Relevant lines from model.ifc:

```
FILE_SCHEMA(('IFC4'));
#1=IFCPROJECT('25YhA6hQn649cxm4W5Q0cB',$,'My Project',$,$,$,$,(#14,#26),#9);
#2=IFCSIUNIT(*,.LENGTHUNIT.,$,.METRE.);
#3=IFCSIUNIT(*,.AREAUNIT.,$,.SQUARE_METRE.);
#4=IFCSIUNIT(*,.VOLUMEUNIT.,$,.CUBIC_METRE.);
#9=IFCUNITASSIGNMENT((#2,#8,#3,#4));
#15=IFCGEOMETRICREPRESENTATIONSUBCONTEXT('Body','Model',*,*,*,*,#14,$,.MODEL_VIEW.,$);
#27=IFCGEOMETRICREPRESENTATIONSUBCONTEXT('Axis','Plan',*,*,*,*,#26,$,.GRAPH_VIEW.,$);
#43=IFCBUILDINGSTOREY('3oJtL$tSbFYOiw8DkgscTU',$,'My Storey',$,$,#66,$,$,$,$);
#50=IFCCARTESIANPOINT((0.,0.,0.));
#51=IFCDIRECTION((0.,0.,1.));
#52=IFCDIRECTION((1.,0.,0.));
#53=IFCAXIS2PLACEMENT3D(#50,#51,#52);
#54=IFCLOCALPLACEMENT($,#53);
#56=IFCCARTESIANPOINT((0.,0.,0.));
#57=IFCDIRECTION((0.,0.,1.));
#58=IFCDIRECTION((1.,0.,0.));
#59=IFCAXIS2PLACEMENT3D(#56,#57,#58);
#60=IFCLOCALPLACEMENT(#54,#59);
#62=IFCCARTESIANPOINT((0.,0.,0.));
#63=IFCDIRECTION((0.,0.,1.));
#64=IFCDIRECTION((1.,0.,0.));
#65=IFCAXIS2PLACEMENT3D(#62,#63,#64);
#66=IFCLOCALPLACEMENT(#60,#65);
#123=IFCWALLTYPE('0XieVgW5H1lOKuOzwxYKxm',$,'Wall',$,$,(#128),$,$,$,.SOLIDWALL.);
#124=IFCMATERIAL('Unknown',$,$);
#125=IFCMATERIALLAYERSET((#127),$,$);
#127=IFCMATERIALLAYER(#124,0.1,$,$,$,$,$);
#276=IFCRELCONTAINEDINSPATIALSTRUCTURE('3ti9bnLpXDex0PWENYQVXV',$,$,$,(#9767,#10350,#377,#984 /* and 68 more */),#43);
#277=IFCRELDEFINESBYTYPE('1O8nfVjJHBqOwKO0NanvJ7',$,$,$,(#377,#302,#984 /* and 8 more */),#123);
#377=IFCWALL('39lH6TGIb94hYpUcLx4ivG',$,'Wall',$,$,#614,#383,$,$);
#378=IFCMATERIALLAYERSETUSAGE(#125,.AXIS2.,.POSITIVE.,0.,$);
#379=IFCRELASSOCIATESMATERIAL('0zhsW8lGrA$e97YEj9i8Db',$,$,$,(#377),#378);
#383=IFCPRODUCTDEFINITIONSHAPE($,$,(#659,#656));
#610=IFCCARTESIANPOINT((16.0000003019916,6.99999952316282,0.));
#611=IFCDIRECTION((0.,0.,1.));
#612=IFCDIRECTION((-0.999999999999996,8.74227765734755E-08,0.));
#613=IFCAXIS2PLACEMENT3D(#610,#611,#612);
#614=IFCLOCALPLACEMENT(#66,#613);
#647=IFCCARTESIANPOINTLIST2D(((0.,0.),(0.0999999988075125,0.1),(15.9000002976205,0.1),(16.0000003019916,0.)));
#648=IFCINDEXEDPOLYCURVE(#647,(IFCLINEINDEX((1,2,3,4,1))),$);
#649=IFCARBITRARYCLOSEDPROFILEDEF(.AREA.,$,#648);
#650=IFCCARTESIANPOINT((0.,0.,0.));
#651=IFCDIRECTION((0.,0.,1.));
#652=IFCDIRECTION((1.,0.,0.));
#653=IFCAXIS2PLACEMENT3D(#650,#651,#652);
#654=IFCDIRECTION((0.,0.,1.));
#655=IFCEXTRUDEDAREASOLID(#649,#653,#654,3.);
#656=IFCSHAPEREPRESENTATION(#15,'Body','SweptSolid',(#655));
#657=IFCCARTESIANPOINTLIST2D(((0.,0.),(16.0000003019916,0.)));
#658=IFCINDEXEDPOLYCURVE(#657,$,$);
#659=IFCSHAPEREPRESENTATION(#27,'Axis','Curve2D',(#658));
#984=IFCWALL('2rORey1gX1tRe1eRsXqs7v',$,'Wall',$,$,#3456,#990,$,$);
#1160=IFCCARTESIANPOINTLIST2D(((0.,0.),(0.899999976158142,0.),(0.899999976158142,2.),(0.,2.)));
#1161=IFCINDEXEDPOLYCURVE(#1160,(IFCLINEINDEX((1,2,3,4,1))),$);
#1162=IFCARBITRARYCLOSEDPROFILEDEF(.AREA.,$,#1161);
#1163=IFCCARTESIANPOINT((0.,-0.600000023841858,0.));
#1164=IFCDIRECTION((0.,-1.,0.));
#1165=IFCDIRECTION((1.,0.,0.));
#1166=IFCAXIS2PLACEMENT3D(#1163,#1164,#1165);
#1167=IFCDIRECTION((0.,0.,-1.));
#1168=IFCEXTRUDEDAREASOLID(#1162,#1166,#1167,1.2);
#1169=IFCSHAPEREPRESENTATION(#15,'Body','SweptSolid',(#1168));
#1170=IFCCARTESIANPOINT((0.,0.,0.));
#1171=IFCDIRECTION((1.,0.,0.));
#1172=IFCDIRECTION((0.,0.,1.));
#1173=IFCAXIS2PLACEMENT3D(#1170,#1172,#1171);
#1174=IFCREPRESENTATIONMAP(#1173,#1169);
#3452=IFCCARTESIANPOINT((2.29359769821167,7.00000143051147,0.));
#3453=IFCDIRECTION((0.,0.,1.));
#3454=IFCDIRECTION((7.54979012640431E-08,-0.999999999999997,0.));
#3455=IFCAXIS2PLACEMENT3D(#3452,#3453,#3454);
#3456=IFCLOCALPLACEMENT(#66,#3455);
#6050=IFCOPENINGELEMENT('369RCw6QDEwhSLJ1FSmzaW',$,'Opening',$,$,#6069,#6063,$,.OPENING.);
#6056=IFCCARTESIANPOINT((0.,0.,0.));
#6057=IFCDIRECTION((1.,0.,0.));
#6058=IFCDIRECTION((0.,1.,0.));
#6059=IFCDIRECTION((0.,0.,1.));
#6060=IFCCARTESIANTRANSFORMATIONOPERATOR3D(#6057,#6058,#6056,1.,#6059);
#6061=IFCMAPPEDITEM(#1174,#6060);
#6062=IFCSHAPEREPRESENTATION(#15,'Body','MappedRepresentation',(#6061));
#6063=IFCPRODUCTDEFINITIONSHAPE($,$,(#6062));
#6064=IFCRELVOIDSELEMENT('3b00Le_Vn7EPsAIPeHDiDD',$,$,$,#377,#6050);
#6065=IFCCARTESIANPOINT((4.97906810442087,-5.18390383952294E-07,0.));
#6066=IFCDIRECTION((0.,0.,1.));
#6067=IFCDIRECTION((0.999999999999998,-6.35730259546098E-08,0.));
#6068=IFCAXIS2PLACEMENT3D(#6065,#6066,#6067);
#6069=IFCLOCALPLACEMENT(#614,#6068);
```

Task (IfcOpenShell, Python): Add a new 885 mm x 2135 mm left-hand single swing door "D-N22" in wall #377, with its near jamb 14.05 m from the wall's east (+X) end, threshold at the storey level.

```python
import numpy as np
import ifcopenshell
import ifcopenshell.api.feature
import ifcopenshell.api.geometry
import ifcopenshell.api.root
import ifcopenshell.api.spatial
import ifcopenshell.geom
import ifcopenshell.util.element
import ifcopenshell.util.placement
import ifcopenshell.util.representation
import ifcopenshell.util.shape
import ifcopenshell.util.unit

model = ifcopenshell.open("model.ifc")
unit_scale = ifcopenshell.util.unit.calculate_unit_scale(model)
settings = ifcopenshell.geom.settings()


def volume(element):
    """Net volume in cubic metres, openings subtracted."""
    shape = ifcopenshell.geom.create_shape(settings, element)
    return ifcopenshell.util.shape.get_volume(shape.geometry)


wall = model.by_id(377)
storey = ifcopenshell.util.element.get_container(wall, ifc_class="IfcBuildingStorey")
context = ifcopenshell.util.representation.get_context(model, "Model", "Body", "MODEL_VIEW")
before = volume(wall)

width, height, from_end, sill = 0.885, 2.135, 14.05, 0.0  # metres

# The wall runs along its own X axis, and the end named is its -X end.
wall_shape = ifcopenshell.geom.create_shape(settings, wall)
x, y, z = ifcopenshell.util.shape.get_vertices(wall_shape.geometry).T
start = x.min() + from_end
face, thickness = float(y.min()), float(y.max() - y.min())
wall_matrix = ifcopenshell.util.placement.get_local_placement(wall.ObjectPlacement)
level = ifcopenshell.util.placement.get_local_placement(storey.ObjectPlacement)[2, 3]


def in_wall(x, y):
    """Placement at x, y metres in the wall's axes, at sill height."""
    matrix = wall_matrix.copy()
    matrix[:, 3] = wall_matrix @ np.array([x / unit_scale, y / unit_scale, 0.0, 1.0])
    matrix[2, 3] = level + sill / unit_scale
    return matrix


# Opening: a box that overshoots both wall faces by 50 mm.
opening = ifcopenshell.api.root.create_entity(model, ifc_class="IfcOpeningElement", predefined_type="OPENING")
box = ifcopenshell.api.geometry.add_wall_representation(
    model, context=context, length=width, height=height, thickness=thickness + 0.1
)
ifcopenshell.api.geometry.assign_representation(model, product=opening, representation=box)
ifcopenshell.api.geometry.edit_object_placement(model, product=opening, matrix=in_wall(start, face - 0.05), is_si=False)
ifcopenshell.api.feature.add_feature(model, feature=opening, element=wall)

door = ifcopenshell.api.root.create_entity(model, ifc_class="IfcDoor", name="D-N22", predefined_type="DOOR")
door.OverallWidth, door.OverallHeight = width / unit_scale, height / unit_scale
door.OperationType = "SINGLE_SWING_LEFT"
body = ifcopenshell.api.geometry.add_door_representation(
    model,
    context=context,
    overall_width=door.OverallWidth,
    overall_height=door.OverallHeight,
    operation_type="SINGLE_SWING_LEFT",
    lining_properties={"LiningDepth": thickness / unit_scale, "ThresholdDepth": thickness / unit_scale},
)
ifcopenshell.api.geometry.assign_representation(model, product=door, representation=body)
ifcopenshell.api.spatial.assign_container(model, products=[door], relating_structure=storey)
ifcopenshell.api.feature.add_filling(model, opening=opening, element=door)

# The lining spans the wall, so the door starts at the wall face.
ifcopenshell.api.geometry.edit_object_placement(model, product=door, matrix=in_wall(start, face), is_si=False)

after = volume(wall)

print(f"wall volume {before:.3f} -> {after:.3f} m3")

model.write("model-out.ifc")
```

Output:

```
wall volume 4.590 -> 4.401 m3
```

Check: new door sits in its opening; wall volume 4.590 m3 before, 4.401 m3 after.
